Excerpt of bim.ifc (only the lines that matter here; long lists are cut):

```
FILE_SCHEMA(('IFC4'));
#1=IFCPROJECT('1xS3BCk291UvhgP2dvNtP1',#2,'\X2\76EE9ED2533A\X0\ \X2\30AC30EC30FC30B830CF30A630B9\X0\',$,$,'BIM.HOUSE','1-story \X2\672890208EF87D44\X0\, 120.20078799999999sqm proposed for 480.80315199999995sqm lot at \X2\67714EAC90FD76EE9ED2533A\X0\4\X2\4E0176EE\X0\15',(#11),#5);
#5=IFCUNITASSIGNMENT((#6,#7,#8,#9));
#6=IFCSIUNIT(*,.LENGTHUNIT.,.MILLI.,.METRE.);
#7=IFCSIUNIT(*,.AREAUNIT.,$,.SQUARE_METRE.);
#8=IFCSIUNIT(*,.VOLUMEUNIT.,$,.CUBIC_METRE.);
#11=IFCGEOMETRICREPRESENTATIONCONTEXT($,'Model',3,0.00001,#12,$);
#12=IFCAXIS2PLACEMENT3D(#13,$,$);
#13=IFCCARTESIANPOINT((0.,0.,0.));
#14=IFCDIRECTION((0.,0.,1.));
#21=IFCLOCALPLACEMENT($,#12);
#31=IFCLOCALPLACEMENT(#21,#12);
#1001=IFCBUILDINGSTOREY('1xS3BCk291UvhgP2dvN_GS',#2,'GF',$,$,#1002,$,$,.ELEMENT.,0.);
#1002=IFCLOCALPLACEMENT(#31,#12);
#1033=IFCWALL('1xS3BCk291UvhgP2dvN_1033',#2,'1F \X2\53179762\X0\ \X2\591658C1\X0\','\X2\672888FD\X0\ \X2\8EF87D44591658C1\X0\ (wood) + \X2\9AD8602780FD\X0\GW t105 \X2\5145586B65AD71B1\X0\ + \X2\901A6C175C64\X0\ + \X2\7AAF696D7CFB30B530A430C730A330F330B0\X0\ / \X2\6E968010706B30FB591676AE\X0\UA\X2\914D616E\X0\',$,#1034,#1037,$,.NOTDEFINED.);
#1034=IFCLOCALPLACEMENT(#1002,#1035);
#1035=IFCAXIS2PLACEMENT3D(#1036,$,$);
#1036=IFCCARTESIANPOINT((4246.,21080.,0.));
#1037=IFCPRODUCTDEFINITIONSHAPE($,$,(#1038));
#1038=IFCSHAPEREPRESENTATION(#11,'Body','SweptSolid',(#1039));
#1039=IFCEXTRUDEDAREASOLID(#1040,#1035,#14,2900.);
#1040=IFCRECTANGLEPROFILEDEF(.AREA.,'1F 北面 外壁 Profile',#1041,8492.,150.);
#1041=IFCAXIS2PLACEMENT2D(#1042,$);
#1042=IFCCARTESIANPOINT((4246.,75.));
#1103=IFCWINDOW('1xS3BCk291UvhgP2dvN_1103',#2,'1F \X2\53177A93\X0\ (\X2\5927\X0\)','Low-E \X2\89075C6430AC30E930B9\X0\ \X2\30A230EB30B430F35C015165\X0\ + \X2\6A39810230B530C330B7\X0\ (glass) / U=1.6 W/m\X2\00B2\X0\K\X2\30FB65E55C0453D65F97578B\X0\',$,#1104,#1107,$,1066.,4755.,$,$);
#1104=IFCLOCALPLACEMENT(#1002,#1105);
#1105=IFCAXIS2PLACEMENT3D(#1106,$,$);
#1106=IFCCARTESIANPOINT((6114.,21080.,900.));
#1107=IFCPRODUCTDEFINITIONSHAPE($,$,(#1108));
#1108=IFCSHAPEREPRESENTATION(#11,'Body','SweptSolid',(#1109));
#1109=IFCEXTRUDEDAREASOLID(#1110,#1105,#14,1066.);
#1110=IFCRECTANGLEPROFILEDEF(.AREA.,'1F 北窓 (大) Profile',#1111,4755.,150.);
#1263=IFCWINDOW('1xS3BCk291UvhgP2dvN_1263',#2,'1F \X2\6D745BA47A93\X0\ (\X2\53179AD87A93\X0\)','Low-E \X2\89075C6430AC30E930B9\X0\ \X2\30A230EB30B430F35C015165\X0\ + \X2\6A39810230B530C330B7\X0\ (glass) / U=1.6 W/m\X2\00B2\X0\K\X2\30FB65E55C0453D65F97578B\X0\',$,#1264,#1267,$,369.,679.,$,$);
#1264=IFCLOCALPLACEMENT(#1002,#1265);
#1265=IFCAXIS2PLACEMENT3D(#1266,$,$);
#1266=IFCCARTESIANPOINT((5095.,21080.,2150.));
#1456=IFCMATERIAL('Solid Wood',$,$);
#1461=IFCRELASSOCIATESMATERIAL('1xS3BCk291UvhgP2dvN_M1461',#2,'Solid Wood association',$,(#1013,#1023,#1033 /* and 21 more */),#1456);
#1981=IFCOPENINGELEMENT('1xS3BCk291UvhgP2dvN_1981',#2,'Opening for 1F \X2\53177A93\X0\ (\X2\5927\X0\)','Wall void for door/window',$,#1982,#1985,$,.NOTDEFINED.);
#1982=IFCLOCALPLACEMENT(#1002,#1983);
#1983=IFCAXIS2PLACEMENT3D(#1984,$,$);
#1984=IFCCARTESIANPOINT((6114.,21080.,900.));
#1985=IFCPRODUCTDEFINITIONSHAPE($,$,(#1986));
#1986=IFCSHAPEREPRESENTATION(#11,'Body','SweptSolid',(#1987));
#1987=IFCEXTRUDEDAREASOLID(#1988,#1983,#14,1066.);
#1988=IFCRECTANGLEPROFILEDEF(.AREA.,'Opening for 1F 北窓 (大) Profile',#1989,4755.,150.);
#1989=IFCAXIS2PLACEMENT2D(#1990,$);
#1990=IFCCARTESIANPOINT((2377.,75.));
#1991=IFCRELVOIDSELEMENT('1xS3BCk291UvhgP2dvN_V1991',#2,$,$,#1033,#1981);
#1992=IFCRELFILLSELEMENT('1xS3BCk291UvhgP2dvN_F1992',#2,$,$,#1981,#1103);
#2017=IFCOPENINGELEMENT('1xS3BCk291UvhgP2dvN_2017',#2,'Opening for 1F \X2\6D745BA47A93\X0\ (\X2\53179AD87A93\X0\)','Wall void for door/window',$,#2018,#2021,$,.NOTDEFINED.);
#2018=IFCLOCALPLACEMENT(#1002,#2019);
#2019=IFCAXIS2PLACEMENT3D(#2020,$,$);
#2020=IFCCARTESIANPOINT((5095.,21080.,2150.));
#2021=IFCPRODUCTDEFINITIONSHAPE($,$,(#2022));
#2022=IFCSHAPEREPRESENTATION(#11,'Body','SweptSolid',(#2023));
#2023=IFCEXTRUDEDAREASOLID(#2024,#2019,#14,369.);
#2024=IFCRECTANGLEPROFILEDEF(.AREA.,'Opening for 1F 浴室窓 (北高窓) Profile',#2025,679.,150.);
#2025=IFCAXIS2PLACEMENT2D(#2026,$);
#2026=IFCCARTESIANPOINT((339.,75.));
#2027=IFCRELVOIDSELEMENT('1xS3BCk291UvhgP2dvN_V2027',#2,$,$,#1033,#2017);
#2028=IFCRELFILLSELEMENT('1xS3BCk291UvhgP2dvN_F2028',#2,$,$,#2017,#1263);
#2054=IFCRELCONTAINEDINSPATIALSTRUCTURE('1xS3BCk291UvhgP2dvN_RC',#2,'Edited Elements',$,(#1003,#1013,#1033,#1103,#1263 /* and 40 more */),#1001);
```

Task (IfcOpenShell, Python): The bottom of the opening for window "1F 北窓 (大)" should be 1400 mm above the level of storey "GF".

```python
import numpy as np
import ifcopenshell
import ifcopenshell.api.geometry
import ifcopenshell.geom
import ifcopenshell.util.element
import ifcopenshell.util.placement
import ifcopenshell.util.shape
import ifcopenshell.util.unit

model = ifcopenshell.open("bim.ifc")
unit_scale = ifcopenshell.util.unit.calculate_unit_scale(model)

window = model.by_id(1103)
opening = window.FillsVoids[0].RelatingOpeningElement
storey = ifcopenshell.util.element.get_container(window, ifc_class="IfcBuildingStorey")
level = ifcopenshell.util.placement.get_local_placement(storey.ObjectPlacement)[2, 3]

# The opening's origin need not be at the sill, so measure its lowest point.
shape = ifcopenshell.geom.create_shape(ifcopenshell.geom.settings(), opening)
bottom = ifcopenshell.util.shape.get_shape_bottom_elevation(shape, shape.geometry) / unit_scale
dz = level + 1.4 / unit_scale - bottom

shift = np.array([0.0, 0.0, dz])
# The window is not placed relative to its opening, so move both.
for product in (opening, window):
    matrix = ifcopenshell.util.placement.get_local_placement(product.ObjectPlacement)
    matrix[:3, 3] += shift
    ifcopenshell.api.geometry.edit_object_placement(model, product=product, matrix=matrix, is_si=False)

print(f"moved by {dz * unit_scale:+.3f} m")

model.write("bim-out.ifc")
```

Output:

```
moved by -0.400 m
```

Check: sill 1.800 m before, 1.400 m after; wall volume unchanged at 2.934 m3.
